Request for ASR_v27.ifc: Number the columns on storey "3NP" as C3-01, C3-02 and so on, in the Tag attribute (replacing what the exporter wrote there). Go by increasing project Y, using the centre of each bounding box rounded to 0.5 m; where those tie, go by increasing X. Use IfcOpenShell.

First a look at what the model holds.

```python
import ifcopenshell
import ifcopenshell.util.element
import ifcopenshell.util.placement

model = ifcopenshell.open("ASR_v27.ifc")
print(model.schema)
storey = next(s for s in model.by_type("IfcBuildingStorey") if s.Name == "3NP")
columns = [e for e in ifcopenshell.util.element.get_decomposition(storey) if e.is_a("IfcColumn")]
for e in sorted(columns, key=lambda e: e.id()):
    origin = ifcopenshell.util.placement.get_local_placement(e.ObjectPlacement)[:3, 3]
    print(e.id(), e.Tag, e.Name, origin.round(2) + 0.0, sep=" | ")
```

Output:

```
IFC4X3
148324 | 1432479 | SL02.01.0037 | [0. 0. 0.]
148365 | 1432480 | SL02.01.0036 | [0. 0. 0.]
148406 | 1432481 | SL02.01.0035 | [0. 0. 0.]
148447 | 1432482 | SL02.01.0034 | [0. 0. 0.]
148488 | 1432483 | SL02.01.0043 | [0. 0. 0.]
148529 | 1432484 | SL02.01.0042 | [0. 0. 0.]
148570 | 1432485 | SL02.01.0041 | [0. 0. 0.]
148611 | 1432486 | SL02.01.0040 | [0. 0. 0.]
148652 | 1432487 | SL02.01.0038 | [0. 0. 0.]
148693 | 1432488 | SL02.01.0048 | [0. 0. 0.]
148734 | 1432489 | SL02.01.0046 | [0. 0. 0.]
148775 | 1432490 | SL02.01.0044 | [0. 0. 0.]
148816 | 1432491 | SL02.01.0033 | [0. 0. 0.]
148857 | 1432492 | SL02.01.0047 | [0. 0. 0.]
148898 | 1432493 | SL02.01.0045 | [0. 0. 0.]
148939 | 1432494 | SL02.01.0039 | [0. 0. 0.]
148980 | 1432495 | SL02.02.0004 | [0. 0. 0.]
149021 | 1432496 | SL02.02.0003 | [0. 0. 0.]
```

```python
import ifcopenshell
import ifcopenshell.geom
import ifcopenshell.util.element
import ifcopenshell.util.shape

model = ifcopenshell.open("ASR_v27.ifc")
settings = ifcopenshell.geom.settings()
settings.set("use-world-coords", True)


def centre(element):
    shape = ifcopenshell.geom.create_shape(settings, element)
    return ifcopenshell.util.shape.get_bbox_centroid(shape.geometry)


storey = next(s for s in model.by_type("IfcBuildingStorey") if s.Name == "3NP")
columns = [e for e in ifcopenshell.util.element.get_decomposition(storey) if e.is_a("IfcColumn")]

# Insertion points can sit at a corner or the storey origin, so sort by the geometry (in metres).
centres = {e: centre(e) for e in columns}
columns.sort(key=lambda e: (round(centres[e][1] / 0.5), centres[e][0]))

for i, e in enumerate(columns, start=1):
    number = f"C3-{i:02d}"
    e.Tag = number
    print(e.id(), number)

model.write("ASR_v27_rev.ifc")
```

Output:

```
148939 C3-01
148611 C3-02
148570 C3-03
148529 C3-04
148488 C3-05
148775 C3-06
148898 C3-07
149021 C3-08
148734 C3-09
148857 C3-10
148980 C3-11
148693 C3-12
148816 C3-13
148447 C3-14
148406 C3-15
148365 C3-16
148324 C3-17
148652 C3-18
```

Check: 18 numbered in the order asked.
